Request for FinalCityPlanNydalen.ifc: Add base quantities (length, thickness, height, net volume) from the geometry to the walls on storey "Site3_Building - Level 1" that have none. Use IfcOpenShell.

First a look at what the model holds.

```python
import ifcopenshell
import ifcopenshell.util.element
import ifcopenshell.util.unit

model = ifcopenshell.open("FinalCityPlanNydalen.ifc")
print(model.schema)
for unit_type in ("LENGTHUNIT", "AREAUNIT", "VOLUMEUNIT"):
    print(unit_type, ifcopenshell.util.unit.calculate_unit_scale(model, unit_type))
storey = next(s for s in model.by_type("IfcBuildingStorey") if s.Name == "Site3_Building - Level 1")
walls = [e for e in ifcopenshell.util.element.get_decomposition(storey) if e.is_a("IfcWall")]
for e in sorted(walls, key=lambda e: e.id()):
    print(e.id(), e.is_a(), e.Name, list(ifcopenshell.util.element.get_psets(e, qtos_only=True)), sep=" | ")
```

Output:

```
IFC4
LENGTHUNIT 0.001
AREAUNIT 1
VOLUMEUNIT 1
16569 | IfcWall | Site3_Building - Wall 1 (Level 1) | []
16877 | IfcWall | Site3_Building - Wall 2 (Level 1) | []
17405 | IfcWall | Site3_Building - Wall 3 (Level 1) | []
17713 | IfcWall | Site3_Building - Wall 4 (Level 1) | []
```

```python
import ifcopenshell
import ifcopenshell.api.pset
import ifcopenshell.geom
import ifcopenshell.util.element
import ifcopenshell.util.shape
import ifcopenshell.util.unit

model = ifcopenshell.open("FinalCityPlanNydalen.ifc")
unit_scale = ifcopenshell.util.unit.calculate_unit_scale(model)
volume_scale = ifcopenshell.util.unit.calculate_unit_scale(model, "VOLUMEUNIT")
settings = ifcopenshell.geom.settings()

storey = next(s for s in model.by_type("IfcBuildingStorey") if s.Name == "Site3_Building - Level 1")
walls = [e for e in ifcopenshell.util.element.get_decomposition(storey) if e.is_a("IfcWall")]

for e in sorted(walls, key=lambda e: e.id()):
    if ifcopenshell.util.element.get_psets(e, qtos_only=True, should_inherit=False):
        continue
    # Geometry comes back in metres, in the element's own axes.
    shape = ifcopenshell.geom.create_shape(settings, e)
    values = {
        "Length": ifcopenshell.util.shape.get_x(shape.geometry) / unit_scale,
        "Width": ifcopenshell.util.shape.get_y(shape.geometry) / unit_scale,
        "Height": ifcopenshell.util.shape.get_z(shape.geometry) / unit_scale,
        "NetVolume": ifcopenshell.util.shape.get_volume(shape.geometry) / volume_scale,
    }
    qto = ifcopenshell.api.pset.add_qto(model, product=e, name="Qto_WallBaseQuantities")
    ifcopenshell.api.pset.edit_qto(model, qto=qto, properties=values)
    print(e.id(), {k: round(v, 3) for k, v in values.items()})

model.write("FinalCityPlanNydalen_edited.ifc")
```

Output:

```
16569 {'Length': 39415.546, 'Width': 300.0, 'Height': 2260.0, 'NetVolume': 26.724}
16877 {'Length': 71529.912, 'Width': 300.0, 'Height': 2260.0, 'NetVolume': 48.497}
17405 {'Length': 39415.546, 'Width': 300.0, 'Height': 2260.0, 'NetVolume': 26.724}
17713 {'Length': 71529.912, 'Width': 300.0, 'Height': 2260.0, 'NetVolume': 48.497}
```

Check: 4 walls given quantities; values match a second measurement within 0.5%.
